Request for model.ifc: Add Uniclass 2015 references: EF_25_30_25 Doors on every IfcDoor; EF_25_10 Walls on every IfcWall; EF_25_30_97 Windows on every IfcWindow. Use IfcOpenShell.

First a look at what the model holds.

```python
import ifcopenshell

model = ifcopenshell.open("model.ifc")
print(model.schema)
print("classifications:", [c.Name for c in model.by_type("IfcClassification")])
for ifc_class in ("IfcDoor", "IfcRoof", "IfcStair", "IfcWall", "IfcWindow"):
    print(ifc_class, len(model.by_type(ifc_class)))
```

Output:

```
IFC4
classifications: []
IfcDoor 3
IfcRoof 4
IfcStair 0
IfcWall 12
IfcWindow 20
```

```python
import ifcopenshell
import ifcopenshell.api.classification

model = ifcopenshell.open("model.ifc")

system = ifcopenshell.api.classification.add_classification(model, classification="Uniclass 2015")

codes = {
    "IfcDoor": ("EF_25_30_25", "Doors"),
    "IfcWall": ("EF_25_10", "Walls"),
    "IfcWindow": ("EF_25_30_97", "Windows"),
}
for ifc_class, (code, name) in codes.items():
    products = model.by_type(ifc_class)
    ifcopenshell.api.classification.add_reference(
        model, products=products, classification=system, identification=code, name=name
    )
    print(code, len(products))

model.write("model_v2.ifc")
```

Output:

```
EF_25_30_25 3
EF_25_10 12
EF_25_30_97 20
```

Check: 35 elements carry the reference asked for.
